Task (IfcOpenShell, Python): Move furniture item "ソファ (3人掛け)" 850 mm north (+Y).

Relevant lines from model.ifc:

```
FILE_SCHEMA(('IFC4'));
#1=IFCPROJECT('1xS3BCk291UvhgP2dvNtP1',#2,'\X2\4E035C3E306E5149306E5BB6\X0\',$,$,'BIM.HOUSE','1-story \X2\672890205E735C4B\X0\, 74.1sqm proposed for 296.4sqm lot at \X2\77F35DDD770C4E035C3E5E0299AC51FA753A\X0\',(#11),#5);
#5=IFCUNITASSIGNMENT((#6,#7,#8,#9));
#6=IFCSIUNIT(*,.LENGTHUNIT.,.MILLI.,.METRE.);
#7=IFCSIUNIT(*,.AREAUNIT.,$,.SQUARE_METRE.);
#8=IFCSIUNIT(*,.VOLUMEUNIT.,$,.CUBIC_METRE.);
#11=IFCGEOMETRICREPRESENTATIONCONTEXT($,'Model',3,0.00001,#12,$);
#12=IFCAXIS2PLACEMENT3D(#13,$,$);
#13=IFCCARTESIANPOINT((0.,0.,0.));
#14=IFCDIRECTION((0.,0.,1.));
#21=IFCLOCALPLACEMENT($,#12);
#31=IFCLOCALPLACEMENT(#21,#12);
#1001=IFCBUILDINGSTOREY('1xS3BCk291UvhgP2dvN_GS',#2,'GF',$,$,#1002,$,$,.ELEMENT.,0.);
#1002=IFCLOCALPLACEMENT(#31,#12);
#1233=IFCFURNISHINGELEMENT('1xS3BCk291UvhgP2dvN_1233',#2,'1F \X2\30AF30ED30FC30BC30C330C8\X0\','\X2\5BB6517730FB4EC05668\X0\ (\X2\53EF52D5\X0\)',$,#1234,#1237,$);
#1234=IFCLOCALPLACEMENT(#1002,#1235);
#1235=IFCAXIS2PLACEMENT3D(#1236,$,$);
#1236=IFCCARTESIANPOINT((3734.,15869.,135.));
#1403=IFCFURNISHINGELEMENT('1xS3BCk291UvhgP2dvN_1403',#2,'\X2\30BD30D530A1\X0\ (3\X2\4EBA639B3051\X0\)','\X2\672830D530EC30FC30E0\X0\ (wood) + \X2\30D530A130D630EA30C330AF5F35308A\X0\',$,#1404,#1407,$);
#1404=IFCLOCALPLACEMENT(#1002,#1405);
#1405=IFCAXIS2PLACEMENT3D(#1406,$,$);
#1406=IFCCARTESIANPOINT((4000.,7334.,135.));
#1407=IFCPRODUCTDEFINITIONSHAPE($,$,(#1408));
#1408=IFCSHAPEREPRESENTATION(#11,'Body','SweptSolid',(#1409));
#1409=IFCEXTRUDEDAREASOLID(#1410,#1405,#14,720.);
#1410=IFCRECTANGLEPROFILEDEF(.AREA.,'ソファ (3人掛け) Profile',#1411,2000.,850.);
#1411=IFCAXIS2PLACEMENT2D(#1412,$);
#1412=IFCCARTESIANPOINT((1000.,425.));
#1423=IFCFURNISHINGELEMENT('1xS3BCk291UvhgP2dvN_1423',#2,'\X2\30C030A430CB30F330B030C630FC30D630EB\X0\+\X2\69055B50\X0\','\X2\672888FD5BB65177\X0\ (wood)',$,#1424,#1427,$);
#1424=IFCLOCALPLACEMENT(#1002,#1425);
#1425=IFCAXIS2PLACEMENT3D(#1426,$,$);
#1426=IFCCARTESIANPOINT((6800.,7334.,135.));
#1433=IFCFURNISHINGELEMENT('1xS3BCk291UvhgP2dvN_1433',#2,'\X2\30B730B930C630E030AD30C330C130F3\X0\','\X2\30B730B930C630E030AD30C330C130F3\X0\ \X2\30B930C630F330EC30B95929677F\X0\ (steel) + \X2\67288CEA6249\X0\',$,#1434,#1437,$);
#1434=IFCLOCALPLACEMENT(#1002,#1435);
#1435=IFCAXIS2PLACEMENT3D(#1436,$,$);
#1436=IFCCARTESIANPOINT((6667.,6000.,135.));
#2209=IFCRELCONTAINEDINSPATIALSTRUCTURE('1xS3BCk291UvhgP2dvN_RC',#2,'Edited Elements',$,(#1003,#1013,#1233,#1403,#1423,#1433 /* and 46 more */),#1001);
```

```python
import ifcopenshell
import ifcopenshell.api.geometry
import ifcopenshell.util.placement

model = ifcopenshell.open("model.ifc")

item = model.by_guid("1xS3BCk291UvhgP2dvN_1403")
matrix = ifcopenshell.util.placement.get_local_placement(item.ObjectPlacement)
matrix[1, 3] += 850.0
ifcopenshell.api.geometry.edit_object_placement(model, product=item, matrix=matrix, is_si=False)

print(ifcopenshell.util.placement.get_local_placement(item.ObjectPlacement).round(3) + 0.0)

model.write("model_updated.ifc")
```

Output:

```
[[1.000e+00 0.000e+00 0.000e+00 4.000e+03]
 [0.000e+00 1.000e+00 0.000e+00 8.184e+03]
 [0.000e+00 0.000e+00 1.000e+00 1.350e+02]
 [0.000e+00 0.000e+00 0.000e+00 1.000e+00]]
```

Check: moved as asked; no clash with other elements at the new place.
